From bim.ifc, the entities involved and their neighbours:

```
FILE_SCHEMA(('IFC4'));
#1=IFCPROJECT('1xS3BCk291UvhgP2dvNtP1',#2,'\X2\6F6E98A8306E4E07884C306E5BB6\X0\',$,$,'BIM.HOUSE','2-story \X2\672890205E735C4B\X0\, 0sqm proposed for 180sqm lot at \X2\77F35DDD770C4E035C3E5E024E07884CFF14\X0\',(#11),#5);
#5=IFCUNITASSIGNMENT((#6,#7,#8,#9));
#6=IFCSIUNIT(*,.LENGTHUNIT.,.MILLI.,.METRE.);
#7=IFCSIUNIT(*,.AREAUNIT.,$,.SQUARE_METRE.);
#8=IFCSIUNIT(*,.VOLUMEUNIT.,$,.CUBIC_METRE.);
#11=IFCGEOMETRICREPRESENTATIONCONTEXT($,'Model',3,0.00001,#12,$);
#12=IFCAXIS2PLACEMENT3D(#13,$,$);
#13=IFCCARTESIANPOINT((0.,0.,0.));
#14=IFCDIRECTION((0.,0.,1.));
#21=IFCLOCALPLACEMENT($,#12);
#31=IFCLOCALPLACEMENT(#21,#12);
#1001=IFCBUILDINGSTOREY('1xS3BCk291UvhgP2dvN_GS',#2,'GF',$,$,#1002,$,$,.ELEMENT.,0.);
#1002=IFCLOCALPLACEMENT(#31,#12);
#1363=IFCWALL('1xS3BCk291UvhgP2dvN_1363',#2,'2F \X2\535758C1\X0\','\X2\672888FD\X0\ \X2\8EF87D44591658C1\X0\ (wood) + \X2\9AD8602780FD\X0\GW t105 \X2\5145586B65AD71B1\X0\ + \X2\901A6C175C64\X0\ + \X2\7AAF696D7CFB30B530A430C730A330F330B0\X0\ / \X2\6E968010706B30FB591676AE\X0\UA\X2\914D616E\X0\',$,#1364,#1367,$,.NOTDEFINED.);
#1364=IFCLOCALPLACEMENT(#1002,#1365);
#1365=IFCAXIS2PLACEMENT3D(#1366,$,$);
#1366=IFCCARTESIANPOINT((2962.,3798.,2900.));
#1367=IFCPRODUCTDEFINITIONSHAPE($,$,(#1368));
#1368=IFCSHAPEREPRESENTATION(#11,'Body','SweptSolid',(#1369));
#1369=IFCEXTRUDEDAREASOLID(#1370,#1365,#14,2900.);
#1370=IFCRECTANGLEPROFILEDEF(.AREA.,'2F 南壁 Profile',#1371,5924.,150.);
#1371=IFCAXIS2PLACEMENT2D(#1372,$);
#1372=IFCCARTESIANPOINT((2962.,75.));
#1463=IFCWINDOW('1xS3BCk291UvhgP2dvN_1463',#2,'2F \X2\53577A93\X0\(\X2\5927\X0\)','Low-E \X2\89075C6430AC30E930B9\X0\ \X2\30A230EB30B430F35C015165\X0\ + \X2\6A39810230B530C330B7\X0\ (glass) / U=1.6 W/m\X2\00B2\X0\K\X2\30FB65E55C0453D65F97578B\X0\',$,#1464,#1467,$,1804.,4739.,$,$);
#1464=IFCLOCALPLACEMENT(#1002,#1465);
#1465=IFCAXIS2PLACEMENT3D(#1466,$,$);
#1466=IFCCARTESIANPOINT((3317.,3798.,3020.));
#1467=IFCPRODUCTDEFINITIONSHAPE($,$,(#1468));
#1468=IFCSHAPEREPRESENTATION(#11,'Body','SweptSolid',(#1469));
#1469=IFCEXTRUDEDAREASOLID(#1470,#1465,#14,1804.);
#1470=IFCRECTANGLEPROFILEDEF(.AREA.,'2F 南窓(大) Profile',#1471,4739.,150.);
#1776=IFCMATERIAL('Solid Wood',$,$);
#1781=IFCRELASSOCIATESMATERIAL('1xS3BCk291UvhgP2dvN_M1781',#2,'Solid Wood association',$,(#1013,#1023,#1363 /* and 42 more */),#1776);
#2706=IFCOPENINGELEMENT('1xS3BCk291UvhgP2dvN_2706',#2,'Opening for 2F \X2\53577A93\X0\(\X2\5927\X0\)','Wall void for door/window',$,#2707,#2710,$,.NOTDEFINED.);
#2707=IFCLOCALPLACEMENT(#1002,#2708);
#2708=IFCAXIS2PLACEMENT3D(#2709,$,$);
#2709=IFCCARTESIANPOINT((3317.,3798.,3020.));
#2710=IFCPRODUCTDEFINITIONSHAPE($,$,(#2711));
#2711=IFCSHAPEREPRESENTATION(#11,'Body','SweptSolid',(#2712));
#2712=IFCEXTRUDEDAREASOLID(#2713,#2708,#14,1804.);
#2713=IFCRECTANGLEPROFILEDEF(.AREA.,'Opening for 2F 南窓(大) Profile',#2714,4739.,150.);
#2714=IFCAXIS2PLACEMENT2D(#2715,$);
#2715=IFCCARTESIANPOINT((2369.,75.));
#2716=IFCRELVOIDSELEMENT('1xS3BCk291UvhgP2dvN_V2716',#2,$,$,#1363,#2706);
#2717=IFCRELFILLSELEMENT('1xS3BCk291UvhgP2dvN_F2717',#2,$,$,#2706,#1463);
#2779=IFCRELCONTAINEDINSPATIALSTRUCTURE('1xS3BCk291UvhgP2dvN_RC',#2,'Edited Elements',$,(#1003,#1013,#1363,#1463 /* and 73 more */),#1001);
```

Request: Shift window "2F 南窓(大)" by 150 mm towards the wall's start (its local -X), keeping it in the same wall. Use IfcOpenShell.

```python
import ifcopenshell
import ifcopenshell.api.geometry
import ifcopenshell.util.placement
import ifcopenshell.util.unit

model = ifcopenshell.open("bim.ifc")
unit_scale = ifcopenshell.util.unit.calculate_unit_scale(model)

window = model.by_guid("1xS3BCk291UvhgP2dvN_1463")
opening = window.FillsVoids[0].RelatingOpeningElement
wall = opening.VoidsElements[0].RelatingBuildingElement

wall_matrix = ifcopenshell.util.placement.get_local_placement(wall.ObjectPlacement)
shift = wall_matrix[:3, 0] * -0.15 / unit_scale
before = ifcopenshell.util.placement.get_local_placement(window.ObjectPlacement)[:3, 3].copy()

# The window is not placed relative to its opening, so move both.
for product in (opening, window):
    matrix = ifcopenshell.util.placement.get_local_placement(product.ObjectPlacement)
    matrix[:3, 3] += shift
    ifcopenshell.api.geometry.edit_object_placement(model, product=product, matrix=matrix, is_si=False)

after = ifcopenshell.util.placement.get_local_placement(window.ObjectPlacement)[:3, 3]
print("window moved by", (after - before).round(3) + 0.0)

model.write("bim_v2.ifc")
```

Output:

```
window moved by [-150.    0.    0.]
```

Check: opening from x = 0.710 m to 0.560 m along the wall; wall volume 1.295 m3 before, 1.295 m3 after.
